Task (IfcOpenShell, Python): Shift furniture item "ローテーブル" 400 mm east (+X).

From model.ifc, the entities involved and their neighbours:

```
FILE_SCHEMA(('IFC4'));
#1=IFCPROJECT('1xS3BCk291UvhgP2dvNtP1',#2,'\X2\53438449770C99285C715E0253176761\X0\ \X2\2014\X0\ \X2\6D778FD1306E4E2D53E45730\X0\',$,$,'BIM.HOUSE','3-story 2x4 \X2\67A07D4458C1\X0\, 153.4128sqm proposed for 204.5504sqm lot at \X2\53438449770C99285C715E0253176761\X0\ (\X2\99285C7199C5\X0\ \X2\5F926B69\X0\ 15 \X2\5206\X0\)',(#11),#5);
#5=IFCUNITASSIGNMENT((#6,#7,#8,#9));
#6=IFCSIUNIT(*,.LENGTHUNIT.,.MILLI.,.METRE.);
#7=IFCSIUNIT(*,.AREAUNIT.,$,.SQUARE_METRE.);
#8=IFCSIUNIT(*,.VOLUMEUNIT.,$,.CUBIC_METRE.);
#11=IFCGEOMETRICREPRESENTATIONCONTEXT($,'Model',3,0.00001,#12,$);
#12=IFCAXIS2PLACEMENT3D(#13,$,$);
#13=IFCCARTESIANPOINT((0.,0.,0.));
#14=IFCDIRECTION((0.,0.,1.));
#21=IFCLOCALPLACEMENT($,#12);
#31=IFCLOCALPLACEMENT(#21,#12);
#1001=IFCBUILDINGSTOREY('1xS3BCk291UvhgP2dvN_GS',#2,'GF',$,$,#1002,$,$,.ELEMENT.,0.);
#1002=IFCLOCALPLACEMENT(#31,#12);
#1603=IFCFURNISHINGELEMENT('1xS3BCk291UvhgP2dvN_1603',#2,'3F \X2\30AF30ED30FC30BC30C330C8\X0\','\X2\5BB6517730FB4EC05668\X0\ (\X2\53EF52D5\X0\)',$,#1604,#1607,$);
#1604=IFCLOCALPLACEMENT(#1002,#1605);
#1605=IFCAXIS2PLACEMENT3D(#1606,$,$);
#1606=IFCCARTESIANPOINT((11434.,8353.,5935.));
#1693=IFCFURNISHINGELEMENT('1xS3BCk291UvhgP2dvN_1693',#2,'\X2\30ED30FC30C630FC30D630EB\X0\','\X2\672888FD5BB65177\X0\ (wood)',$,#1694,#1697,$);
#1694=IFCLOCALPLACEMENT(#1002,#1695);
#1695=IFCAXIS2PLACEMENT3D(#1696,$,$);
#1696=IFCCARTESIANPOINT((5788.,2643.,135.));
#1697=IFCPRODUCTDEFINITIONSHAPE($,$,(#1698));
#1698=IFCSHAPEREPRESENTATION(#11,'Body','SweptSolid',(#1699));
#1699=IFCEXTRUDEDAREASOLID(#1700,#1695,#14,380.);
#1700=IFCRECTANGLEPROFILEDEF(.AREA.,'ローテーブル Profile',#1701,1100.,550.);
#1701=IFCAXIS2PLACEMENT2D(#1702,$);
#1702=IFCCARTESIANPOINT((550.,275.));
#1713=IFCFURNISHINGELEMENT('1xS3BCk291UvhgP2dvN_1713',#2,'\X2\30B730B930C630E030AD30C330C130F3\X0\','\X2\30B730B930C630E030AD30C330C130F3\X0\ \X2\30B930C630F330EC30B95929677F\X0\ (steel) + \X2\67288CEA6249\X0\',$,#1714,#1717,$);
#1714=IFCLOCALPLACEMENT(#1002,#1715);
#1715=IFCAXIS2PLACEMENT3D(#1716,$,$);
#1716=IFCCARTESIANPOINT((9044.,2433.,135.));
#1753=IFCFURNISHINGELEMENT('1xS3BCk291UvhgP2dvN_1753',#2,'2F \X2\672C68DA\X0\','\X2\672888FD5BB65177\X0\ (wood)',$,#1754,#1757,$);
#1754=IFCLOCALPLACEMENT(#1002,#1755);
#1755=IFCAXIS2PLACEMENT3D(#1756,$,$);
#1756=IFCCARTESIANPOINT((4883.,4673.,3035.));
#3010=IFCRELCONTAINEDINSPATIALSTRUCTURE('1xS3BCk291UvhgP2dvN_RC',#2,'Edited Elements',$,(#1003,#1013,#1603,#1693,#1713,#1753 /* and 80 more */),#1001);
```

```python
import ifcopenshell
import ifcopenshell.api.geometry
import ifcopenshell.util.placement
import ifcopenshell.util.unit

model = ifcopenshell.open("model.ifc")
unit_scale = ifcopenshell.util.unit.calculate_unit_scale(model)

item = model.by_guid("1xS3BCk291UvhgP2dvN_1693")
matrix = ifcopenshell.util.placement.get_local_placement(item.ObjectPlacement)
matrix[0, 3] += 0.4 / unit_scale
ifcopenshell.api.geometry.edit_object_placement(model, product=item, matrix=matrix, is_si=False)

print(ifcopenshell.util.placement.get_local_placement(item.ObjectPlacement).round(3) + 0.0)

model.write("model_rev.ifc")
```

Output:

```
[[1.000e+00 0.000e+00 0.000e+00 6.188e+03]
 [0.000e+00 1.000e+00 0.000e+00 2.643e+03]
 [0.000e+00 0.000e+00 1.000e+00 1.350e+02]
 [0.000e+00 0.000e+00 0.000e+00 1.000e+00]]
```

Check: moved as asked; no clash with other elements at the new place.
